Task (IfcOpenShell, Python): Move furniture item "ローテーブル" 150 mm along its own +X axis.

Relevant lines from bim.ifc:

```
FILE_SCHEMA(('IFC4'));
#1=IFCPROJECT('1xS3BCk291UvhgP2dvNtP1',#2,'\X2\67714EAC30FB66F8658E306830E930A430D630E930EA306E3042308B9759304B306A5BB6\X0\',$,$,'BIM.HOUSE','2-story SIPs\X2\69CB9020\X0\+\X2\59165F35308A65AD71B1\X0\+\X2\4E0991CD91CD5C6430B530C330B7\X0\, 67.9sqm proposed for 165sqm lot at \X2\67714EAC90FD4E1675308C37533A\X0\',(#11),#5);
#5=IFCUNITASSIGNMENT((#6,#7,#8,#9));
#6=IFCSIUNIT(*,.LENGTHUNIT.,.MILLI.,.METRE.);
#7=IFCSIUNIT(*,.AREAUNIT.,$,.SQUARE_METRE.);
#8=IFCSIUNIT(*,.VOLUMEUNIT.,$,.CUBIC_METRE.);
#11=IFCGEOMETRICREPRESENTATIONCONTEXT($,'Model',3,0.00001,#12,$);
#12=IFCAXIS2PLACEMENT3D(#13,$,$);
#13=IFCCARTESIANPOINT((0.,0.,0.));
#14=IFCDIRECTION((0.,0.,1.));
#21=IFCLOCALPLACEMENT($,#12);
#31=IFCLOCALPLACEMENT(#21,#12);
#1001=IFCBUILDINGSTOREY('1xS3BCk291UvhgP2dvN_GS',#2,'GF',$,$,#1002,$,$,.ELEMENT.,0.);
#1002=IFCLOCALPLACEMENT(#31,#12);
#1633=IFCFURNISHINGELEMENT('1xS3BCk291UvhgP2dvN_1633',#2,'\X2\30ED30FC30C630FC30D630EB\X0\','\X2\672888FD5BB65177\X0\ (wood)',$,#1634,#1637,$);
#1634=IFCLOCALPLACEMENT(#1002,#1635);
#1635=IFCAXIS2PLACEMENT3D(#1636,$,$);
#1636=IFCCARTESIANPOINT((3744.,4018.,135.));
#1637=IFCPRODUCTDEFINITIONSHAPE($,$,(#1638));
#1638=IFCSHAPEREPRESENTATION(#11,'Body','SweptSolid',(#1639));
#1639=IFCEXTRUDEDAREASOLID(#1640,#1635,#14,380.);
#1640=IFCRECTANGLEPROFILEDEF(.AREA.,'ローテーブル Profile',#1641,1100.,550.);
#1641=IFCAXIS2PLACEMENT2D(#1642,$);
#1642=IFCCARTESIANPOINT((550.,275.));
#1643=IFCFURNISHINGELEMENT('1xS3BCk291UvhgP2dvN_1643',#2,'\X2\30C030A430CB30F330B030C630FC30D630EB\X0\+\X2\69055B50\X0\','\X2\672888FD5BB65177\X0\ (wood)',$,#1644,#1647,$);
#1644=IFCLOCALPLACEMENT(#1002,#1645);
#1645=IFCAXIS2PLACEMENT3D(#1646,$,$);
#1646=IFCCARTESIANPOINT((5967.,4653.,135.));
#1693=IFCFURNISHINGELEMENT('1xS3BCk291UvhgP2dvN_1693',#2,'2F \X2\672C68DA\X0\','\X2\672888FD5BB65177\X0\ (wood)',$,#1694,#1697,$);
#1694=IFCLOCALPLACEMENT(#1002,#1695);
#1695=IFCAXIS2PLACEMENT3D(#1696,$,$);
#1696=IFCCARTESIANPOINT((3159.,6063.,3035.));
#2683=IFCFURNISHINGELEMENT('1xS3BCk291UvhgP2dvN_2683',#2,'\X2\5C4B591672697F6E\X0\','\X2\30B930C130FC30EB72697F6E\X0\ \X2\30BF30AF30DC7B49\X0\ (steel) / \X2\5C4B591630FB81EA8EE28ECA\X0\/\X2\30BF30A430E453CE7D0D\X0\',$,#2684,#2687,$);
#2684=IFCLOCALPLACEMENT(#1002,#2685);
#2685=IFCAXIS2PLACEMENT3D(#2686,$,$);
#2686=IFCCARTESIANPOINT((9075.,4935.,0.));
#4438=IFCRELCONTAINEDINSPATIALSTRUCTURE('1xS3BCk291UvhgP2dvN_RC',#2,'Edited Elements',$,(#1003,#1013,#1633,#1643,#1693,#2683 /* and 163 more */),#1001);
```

```python
import ifcopenshell
import ifcopenshell.api.geometry
import ifcopenshell.util.placement

model = ifcopenshell.open("bim.ifc")

item = model.by_guid("1xS3BCk291UvhgP2dvN_1633")
matrix = ifcopenshell.util.placement.get_local_placement(item.ObjectPlacement)
matrix[:3, 3] += matrix[:3, 0] * 150.0
ifcopenshell.api.geometry.edit_object_placement(model, product=item, matrix=matrix, is_si=False)

print(ifcopenshell.util.placement.get_local_placement(item.ObjectPlacement).round(3) + 0.0)

model.write("bim_updated.ifc")
```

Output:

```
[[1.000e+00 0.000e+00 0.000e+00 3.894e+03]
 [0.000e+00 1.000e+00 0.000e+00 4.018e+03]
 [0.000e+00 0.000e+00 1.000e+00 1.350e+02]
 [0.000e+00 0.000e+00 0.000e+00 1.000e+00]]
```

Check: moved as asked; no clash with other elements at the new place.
